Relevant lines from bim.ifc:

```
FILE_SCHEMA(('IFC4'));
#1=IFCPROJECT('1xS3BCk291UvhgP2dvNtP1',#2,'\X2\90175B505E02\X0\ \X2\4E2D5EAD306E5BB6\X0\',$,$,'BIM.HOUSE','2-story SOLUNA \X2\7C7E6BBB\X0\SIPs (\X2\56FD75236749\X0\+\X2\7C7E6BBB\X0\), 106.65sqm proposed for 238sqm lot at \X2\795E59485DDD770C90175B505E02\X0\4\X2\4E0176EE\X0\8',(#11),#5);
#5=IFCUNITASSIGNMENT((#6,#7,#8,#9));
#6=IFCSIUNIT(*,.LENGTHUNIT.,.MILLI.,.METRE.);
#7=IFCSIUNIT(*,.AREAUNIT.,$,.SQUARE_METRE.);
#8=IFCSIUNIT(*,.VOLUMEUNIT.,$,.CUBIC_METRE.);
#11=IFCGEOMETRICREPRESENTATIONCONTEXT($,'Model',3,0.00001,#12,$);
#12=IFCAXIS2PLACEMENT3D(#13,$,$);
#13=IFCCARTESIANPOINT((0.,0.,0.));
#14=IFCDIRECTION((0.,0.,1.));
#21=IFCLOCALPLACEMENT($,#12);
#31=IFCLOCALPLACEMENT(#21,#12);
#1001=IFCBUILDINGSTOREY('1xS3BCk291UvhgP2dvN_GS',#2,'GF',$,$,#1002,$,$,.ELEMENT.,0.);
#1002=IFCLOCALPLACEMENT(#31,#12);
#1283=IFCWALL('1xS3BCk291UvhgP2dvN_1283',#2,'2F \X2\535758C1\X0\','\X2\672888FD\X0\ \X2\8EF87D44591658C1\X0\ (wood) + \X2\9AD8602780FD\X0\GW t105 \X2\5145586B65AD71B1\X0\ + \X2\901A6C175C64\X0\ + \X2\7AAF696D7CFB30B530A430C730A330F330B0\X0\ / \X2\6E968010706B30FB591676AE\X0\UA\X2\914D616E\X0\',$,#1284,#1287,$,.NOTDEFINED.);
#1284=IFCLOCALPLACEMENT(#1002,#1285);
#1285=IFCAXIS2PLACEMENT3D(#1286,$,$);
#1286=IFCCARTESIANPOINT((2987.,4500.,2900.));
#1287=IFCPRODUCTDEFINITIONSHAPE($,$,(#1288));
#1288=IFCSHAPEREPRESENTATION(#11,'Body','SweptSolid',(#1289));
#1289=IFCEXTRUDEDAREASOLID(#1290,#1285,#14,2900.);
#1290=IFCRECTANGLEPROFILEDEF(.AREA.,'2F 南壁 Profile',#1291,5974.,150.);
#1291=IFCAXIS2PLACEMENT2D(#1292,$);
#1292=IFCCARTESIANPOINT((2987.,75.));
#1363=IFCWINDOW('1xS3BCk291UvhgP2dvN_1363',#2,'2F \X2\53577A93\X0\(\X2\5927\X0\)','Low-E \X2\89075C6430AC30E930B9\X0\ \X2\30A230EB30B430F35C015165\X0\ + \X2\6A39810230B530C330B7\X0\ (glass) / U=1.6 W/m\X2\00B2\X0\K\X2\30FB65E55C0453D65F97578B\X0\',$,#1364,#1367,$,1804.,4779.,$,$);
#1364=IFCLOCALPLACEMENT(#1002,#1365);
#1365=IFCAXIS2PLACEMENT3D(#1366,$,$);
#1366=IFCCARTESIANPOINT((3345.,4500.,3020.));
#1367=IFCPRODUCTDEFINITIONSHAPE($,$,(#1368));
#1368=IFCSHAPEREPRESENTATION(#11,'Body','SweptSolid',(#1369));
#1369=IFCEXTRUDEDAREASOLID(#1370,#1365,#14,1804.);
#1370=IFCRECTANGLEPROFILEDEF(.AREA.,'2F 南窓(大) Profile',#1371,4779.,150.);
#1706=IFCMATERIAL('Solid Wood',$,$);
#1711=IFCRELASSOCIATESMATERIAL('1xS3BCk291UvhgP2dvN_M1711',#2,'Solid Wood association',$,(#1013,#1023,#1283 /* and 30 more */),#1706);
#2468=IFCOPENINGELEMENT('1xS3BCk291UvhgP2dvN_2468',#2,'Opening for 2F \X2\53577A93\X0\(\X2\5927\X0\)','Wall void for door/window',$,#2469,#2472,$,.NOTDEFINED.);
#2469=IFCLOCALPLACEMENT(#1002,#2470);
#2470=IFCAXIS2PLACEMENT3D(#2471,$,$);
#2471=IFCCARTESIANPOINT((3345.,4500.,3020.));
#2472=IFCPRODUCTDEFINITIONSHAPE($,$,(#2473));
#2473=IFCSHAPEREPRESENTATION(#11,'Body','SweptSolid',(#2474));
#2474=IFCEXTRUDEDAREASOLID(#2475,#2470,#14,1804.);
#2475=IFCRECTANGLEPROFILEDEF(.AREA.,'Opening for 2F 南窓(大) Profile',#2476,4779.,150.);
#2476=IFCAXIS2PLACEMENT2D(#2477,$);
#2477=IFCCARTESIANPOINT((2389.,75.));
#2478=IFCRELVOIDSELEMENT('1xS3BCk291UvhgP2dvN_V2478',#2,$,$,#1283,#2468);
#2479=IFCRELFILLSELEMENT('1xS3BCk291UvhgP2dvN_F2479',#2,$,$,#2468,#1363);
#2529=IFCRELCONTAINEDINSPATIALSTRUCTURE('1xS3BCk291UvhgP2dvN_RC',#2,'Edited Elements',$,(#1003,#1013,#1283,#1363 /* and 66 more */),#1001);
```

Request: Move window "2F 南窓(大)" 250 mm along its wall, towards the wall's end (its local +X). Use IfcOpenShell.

```python
import ifcopenshell
import ifcopenshell.api.geometry
import ifcopenshell.util.placement
import ifcopenshell.util.unit

model = ifcopenshell.open("bim.ifc")
unit_scale = ifcopenshell.util.unit.calculate_unit_scale(model)

window = model.by_guid("1xS3BCk291UvhgP2dvN_1363")
opening = window.FillsVoids[0].RelatingOpeningElement
wall = opening.VoidsElements[0].RelatingBuildingElement

wall_matrix = ifcopenshell.util.placement.get_local_placement(wall.ObjectPlacement)
shift = wall_matrix[:3, 0] * 0.25 / unit_scale
before = ifcopenshell.util.placement.get_local_placement(window.ObjectPlacement)[:3, 3].copy()

# The window is not placed relative to its opening, so move both.
for product in (opening, window):
    matrix = ifcopenshell.util.placement.get_local_placement(product.ObjectPlacement)
    matrix[:3, 3] += shift
    ifcopenshell.api.geometry.edit_object_placement(model, product=product, matrix=matrix, is_si=False)

after = ifcopenshell.util.placement.get_local_placement(window.ObjectPlacement)[:3, 3]
print("window moved by", (after - before).round(3) + 0.0)

model.write("bim_v2.ifc")
```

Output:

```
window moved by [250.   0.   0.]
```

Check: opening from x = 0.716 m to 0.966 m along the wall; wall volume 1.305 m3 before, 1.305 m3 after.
